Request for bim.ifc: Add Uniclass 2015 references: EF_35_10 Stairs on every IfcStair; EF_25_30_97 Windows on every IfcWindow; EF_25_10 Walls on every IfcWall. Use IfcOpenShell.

First a look at what the model holds.

```python
import ifcopenshell

model = ifcopenshell.open("bim.ifc")
print(model.schema)
print("classifications:", [c.Name for c in model.by_type("IfcClassification")])
for ifc_class in ("IfcDoor", "IfcRoof", "IfcStair", "IfcWall", "IfcWindow"):
    print(ifc_class, len(model.by_type(ifc_class)))
```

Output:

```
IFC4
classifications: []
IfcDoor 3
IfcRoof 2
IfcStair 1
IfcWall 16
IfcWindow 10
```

```python
import ifcopenshell
import ifcopenshell.api.classification

model = ifcopenshell.open("bim.ifc")

system = ifcopenshell.api.classification.add_classification(model, classification="Uniclass 2015")

codes = {
    "IfcStair": ("EF_35_10", "Stairs"),
    "IfcWindow": ("EF_25_30_97", "Windows"),
    "IfcWall": ("EF_25_10", "Walls"),
}
for ifc_class, (code, name) in codes.items():
    products = model.by_type(ifc_class)
    ifcopenshell.api.classification.add_reference(
        model, products=products, classification=system, identification=code, name=name
    )
    print(code, len(products))

model.write("bim-out.ifc")
```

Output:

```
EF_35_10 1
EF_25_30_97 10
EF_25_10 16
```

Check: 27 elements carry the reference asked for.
